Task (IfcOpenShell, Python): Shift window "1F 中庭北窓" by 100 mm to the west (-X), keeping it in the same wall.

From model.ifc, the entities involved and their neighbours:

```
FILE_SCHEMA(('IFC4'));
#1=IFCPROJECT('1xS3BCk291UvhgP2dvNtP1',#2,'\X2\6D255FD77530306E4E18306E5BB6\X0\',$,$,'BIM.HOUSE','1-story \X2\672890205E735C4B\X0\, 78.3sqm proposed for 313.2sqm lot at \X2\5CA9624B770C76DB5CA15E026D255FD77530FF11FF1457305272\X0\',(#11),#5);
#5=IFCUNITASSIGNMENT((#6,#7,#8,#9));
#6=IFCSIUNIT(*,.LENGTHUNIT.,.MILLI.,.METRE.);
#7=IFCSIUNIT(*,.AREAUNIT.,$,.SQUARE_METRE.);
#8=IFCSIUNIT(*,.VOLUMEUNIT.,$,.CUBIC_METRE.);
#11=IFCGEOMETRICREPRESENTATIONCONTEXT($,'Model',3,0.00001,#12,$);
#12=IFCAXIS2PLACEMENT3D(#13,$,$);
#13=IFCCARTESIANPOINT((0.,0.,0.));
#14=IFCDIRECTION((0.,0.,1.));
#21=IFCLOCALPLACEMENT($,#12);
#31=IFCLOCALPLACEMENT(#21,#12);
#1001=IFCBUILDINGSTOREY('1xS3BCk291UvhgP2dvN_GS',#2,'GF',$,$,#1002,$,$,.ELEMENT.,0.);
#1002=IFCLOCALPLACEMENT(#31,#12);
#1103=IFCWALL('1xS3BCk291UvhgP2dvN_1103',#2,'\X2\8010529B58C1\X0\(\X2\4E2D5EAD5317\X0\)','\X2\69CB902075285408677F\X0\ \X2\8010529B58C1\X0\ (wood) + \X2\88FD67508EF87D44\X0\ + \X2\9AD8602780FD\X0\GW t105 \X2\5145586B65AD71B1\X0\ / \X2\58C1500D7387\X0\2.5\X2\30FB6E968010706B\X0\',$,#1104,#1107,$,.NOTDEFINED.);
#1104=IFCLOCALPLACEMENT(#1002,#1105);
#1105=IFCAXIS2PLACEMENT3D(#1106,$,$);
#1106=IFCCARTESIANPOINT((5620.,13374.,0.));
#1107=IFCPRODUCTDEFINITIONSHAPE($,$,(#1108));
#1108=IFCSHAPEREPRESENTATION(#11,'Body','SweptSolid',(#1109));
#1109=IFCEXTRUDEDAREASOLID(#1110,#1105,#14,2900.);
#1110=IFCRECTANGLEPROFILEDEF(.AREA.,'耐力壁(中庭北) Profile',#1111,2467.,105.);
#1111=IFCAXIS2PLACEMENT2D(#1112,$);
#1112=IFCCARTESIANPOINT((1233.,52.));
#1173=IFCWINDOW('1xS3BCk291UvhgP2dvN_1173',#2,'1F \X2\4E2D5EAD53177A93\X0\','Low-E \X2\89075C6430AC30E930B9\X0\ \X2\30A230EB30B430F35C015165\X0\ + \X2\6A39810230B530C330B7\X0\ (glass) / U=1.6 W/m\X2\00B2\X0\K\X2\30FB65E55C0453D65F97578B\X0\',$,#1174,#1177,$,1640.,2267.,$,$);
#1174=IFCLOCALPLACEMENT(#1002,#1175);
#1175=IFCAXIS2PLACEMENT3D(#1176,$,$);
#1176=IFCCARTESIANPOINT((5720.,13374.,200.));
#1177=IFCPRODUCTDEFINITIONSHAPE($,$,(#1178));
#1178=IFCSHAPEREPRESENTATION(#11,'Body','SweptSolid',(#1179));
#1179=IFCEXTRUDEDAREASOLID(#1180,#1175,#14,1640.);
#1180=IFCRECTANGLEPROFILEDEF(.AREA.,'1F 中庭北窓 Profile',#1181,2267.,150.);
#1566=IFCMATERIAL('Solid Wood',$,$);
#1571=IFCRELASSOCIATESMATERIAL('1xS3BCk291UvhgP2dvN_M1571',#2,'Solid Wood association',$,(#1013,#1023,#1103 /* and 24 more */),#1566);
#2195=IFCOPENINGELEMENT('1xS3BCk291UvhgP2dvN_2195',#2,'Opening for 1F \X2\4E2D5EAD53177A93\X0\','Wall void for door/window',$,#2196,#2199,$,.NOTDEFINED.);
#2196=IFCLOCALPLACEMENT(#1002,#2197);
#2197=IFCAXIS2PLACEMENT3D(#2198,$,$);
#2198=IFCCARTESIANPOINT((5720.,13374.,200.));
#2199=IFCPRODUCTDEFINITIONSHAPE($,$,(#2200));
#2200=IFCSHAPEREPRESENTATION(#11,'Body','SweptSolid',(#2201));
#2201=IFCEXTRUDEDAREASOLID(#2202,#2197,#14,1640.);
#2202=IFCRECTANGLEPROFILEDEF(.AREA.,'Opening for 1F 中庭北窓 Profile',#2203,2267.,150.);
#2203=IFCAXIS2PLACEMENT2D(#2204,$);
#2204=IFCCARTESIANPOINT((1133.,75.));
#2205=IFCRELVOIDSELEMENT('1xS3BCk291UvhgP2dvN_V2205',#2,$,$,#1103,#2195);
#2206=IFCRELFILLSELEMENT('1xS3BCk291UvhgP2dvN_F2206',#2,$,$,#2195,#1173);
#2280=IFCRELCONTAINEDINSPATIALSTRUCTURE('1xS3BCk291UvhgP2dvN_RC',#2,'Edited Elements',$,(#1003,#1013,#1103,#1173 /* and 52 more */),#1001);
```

```python
import ifcopenshell
import ifcopenshell.api.geometry
import ifcopenshell.util.placement
import ifcopenshell.util.unit

model = ifcopenshell.open("model.ifc")
unit_scale = ifcopenshell.util.unit.calculate_unit_scale(model)

window = model.by_guid("1xS3BCk291UvhgP2dvN_1173")
opening = window.FillsVoids[0].RelatingOpeningElement
wall = opening.VoidsElements[0].RelatingBuildingElement

wall_matrix = ifcopenshell.util.placement.get_local_placement(wall.ObjectPlacement)
shift = wall_matrix[:3, 0] * -0.1 / unit_scale
before = ifcopenshell.util.placement.get_local_placement(window.ObjectPlacement)[:3, 3].copy()

# The window is not placed relative to its opening, so move both.
for product in (opening, window):
    matrix = ifcopenshell.util.placement.get_local_placement(product.ObjectPlacement)
    matrix[:3, 3] += shift
    ifcopenshell.api.geometry.edit_object_placement(model, product=product, matrix=matrix, is_si=False)

after = ifcopenshell.util.placement.get_local_placement(window.ObjectPlacement)[:3, 3]
print("window moved by", (after - before).round(3) + 0.0)

model.write("model-out.ifc")
```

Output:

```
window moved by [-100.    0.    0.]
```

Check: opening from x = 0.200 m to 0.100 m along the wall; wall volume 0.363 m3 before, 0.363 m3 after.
